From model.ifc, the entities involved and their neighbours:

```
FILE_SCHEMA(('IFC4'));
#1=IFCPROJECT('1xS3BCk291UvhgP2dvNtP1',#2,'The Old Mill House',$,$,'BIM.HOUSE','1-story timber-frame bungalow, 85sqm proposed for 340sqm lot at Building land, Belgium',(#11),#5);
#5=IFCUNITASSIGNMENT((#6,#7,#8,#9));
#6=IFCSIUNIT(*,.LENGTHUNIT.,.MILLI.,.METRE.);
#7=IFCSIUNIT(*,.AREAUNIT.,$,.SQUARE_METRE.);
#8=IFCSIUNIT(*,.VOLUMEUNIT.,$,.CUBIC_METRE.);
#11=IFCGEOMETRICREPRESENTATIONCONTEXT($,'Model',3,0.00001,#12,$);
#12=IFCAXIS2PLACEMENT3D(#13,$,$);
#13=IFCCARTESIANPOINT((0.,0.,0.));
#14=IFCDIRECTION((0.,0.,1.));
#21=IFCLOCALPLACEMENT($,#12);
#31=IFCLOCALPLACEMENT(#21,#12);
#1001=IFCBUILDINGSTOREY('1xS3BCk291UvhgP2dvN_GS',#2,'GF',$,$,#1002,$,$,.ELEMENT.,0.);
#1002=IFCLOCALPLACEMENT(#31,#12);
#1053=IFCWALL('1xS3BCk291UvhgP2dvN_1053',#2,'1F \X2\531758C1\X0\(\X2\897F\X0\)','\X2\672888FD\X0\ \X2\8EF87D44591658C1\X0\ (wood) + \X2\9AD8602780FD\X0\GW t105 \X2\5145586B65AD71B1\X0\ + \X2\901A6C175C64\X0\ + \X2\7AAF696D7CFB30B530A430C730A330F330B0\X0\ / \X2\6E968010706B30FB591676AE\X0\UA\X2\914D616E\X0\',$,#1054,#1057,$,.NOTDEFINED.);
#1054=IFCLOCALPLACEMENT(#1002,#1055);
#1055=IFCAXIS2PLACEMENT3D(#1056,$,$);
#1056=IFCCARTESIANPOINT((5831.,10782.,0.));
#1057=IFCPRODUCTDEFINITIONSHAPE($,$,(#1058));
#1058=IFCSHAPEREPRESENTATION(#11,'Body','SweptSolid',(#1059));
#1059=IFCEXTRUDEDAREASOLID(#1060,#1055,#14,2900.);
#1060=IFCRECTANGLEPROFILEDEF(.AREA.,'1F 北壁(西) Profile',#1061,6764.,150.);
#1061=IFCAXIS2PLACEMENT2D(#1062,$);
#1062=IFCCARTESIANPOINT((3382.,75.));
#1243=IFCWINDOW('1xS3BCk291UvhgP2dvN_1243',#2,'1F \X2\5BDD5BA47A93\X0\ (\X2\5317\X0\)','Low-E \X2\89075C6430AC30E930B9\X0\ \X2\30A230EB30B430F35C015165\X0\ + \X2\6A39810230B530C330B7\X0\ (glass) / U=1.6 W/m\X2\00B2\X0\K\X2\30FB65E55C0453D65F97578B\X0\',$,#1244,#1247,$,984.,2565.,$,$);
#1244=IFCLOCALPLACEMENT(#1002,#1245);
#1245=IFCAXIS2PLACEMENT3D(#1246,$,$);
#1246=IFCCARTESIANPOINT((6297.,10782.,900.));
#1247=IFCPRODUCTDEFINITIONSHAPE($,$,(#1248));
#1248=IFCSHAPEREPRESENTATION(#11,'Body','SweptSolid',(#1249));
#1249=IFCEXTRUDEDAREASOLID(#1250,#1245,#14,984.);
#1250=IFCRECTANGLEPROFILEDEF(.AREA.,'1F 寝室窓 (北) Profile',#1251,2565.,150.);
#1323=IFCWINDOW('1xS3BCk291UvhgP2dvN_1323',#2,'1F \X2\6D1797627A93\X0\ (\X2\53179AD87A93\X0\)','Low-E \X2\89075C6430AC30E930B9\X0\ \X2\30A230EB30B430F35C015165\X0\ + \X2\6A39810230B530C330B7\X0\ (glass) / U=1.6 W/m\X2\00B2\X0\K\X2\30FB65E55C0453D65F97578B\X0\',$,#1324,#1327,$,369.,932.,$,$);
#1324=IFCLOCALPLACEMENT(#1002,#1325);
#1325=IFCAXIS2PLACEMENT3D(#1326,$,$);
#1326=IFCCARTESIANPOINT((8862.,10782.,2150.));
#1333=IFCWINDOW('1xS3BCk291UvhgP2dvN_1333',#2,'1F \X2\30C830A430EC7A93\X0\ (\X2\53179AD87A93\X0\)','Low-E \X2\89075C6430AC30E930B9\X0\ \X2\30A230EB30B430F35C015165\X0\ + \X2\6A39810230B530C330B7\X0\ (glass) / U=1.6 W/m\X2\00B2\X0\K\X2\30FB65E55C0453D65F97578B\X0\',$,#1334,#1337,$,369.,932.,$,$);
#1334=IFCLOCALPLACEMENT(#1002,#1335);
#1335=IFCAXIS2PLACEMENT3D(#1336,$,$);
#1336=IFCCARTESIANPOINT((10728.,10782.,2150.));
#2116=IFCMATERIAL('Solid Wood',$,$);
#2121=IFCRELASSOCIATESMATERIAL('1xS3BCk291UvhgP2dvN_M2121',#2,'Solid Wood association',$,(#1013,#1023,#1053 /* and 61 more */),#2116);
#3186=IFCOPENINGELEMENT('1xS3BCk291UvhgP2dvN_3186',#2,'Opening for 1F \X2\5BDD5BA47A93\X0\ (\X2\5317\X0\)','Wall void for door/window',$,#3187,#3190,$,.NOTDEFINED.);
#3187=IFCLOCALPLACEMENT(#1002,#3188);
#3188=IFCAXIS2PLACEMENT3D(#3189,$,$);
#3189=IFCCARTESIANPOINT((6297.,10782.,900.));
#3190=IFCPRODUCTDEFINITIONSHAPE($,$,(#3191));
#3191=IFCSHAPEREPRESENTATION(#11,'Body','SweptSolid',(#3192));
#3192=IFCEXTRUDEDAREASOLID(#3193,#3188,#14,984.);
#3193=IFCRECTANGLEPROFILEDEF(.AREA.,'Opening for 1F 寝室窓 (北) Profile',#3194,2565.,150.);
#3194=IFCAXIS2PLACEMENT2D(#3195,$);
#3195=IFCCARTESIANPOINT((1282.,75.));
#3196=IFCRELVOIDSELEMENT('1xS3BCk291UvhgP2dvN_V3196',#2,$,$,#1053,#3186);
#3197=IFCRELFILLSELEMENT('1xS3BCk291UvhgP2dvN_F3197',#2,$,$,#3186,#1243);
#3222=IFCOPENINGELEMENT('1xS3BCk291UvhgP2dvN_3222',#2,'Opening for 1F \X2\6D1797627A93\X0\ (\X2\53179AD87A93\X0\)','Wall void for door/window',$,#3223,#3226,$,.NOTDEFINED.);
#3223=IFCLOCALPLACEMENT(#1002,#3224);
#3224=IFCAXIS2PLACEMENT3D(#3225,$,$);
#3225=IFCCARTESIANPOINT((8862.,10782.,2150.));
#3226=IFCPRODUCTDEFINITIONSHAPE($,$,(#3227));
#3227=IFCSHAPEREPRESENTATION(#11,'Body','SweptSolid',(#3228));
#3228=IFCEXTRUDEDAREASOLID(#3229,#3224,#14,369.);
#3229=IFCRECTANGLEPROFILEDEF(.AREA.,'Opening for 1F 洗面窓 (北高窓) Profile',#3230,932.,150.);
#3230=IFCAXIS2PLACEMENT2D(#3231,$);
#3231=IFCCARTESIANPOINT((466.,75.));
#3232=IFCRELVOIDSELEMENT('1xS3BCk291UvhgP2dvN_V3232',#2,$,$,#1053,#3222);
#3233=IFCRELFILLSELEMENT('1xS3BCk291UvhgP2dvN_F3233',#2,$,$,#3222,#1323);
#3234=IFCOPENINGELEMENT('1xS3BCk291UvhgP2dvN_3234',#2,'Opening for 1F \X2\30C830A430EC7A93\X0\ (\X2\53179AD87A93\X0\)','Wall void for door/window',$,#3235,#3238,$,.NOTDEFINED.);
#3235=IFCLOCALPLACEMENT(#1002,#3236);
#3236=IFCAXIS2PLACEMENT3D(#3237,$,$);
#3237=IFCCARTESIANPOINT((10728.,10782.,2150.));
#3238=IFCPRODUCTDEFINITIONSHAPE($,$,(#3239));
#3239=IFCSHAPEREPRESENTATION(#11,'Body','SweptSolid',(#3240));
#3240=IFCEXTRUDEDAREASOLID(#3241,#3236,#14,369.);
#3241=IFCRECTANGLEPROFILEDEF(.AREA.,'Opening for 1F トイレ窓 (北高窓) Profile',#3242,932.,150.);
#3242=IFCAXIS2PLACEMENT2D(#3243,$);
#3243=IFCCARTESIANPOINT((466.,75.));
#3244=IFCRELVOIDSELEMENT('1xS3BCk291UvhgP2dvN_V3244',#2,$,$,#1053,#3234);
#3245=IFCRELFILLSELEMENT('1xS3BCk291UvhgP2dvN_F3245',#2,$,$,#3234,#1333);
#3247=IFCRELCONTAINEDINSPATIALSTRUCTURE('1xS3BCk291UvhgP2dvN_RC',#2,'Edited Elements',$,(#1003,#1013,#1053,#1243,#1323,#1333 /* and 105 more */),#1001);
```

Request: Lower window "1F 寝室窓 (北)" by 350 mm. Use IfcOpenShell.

```python
import numpy as np
import ifcopenshell
import ifcopenshell.api.geometry
import ifcopenshell.util.placement
import ifcopenshell.util.unit

model = ifcopenshell.open("model.ifc")
unit_scale = ifcopenshell.util.unit.calculate_unit_scale(model)

window = model.by_id(1243)
opening = window.FillsVoids[0].RelatingOpeningElement
dz = -0.35 / unit_scale

shift = np.array([0.0, 0.0, dz])
# The window is not placed relative to its opening, so move both.
for product in (opening, window):
    matrix = ifcopenshell.util.placement.get_local_placement(product.ObjectPlacement)
    matrix[:3, 3] += shift
    ifcopenshell.api.geometry.edit_object_placement(model, product=product, matrix=matrix, is_si=False)

print(f"moved by {dz * unit_scale:+.3f} m")

model.write("model-out.ifc")
```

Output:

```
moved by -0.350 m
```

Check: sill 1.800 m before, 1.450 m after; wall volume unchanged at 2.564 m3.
